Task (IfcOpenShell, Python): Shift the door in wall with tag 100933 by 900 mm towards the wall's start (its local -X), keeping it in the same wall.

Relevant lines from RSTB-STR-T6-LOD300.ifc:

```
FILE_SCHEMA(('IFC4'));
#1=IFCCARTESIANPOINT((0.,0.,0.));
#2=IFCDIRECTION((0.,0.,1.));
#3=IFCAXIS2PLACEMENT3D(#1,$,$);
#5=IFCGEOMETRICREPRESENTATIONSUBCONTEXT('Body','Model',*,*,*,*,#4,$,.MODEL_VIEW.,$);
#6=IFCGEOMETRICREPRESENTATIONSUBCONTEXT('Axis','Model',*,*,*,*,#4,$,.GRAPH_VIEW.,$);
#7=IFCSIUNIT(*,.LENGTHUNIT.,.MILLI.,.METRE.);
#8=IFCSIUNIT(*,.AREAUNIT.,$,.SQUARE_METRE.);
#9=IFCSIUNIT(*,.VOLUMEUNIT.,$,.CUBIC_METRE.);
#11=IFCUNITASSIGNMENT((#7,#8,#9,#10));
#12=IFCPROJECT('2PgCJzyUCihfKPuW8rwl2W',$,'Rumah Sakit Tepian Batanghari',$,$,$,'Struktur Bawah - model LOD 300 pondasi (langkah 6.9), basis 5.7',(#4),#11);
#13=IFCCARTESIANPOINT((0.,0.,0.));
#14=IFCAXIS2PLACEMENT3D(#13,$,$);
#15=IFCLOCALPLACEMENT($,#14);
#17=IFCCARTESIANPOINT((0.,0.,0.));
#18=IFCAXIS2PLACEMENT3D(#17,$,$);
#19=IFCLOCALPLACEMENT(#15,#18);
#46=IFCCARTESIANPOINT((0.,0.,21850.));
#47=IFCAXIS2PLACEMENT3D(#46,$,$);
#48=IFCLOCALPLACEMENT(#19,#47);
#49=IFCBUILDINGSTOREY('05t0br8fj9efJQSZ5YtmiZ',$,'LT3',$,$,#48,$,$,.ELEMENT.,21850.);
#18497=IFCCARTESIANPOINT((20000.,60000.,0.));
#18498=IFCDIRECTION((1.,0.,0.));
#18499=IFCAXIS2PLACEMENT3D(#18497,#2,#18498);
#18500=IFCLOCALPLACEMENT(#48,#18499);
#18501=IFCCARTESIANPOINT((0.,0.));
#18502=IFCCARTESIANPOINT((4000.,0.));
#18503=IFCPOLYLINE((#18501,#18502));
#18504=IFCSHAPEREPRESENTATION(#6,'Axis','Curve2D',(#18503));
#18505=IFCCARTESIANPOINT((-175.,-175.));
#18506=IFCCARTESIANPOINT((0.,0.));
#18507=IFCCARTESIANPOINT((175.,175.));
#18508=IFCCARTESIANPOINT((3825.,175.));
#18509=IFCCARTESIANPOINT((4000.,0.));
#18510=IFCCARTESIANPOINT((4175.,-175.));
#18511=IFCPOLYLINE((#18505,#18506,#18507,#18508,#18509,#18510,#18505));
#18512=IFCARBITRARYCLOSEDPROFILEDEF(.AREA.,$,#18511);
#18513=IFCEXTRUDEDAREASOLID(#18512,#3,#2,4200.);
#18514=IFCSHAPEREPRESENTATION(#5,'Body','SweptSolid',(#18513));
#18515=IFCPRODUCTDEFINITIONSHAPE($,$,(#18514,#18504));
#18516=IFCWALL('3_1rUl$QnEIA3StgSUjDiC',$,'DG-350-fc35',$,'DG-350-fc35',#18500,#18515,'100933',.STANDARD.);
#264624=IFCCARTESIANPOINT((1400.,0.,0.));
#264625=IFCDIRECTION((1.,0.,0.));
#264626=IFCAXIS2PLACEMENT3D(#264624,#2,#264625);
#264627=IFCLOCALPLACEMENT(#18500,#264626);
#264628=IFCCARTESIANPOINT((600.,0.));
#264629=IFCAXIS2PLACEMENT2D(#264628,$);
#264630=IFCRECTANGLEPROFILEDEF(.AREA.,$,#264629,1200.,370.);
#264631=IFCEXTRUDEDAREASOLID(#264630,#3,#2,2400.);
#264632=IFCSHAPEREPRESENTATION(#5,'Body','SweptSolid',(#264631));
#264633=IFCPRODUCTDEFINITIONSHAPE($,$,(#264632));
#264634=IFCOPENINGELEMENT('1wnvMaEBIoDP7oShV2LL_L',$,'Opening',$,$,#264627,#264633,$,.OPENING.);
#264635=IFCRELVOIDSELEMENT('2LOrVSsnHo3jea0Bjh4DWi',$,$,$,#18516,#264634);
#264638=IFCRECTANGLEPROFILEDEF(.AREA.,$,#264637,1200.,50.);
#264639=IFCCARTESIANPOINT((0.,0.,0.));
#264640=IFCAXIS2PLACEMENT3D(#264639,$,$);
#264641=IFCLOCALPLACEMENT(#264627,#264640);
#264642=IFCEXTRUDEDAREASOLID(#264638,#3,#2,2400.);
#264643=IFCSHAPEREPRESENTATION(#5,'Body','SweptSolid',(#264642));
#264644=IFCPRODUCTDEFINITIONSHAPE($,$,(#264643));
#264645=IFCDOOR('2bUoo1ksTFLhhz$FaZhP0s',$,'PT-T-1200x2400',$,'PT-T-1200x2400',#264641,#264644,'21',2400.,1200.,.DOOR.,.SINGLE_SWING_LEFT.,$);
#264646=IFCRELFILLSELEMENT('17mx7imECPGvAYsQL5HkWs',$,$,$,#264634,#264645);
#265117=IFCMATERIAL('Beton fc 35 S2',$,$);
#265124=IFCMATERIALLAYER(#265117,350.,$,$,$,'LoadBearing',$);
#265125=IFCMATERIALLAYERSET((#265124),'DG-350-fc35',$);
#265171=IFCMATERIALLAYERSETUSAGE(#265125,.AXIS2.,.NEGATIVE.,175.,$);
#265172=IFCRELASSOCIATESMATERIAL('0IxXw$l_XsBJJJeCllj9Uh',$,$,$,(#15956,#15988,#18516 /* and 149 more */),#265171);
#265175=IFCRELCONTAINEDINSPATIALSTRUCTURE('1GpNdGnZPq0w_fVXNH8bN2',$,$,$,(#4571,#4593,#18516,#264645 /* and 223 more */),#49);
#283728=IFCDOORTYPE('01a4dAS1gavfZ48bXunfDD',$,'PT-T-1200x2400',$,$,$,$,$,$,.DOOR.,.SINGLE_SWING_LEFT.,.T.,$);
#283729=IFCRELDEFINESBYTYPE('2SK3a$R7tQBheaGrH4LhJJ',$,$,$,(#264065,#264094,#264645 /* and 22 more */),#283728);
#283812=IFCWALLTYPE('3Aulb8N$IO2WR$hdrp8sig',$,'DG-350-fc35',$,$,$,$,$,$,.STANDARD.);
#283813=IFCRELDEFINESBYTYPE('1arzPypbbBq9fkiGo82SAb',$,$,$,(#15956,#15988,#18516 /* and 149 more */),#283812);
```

```python
import ifcopenshell
import ifcopenshell.api.geometry
import ifcopenshell.util.placement
import ifcopenshell.util.unit

model = ifcopenshell.open("RSTB-STR-T6-LOD300.ifc")
unit_scale = ifcopenshell.util.unit.calculate_unit_scale(model)

door = model.by_id(264645)
opening = door.FillsVoids[0].RelatingOpeningElement
wall = opening.VoidsElements[0].RelatingBuildingElement

wall_matrix = ifcopenshell.util.placement.get_local_placement(wall.ObjectPlacement)
shift = wall_matrix[:3, 0] * -0.9 / unit_scale
before = ifcopenshell.util.placement.get_local_placement(door.ObjectPlacement)[:3, 3].copy()

# The door is placed relative to its opening, so it follows when the opening moves.
matrix = ifcopenshell.util.placement.get_local_placement(opening.ObjectPlacement)
matrix[:3, 3] += shift
ifcopenshell.api.geometry.edit_object_placement(
    model, product=opening, matrix=matrix, is_si=False, should_transform_children=True
)

after = ifcopenshell.util.placement.get_local_placement(door.ObjectPlacement)[:3, 3]
print("door moved by", (after - before).round(3) + 0.0)

model.write("RSTB-STR-T6-LOD300_v2.ifc")
```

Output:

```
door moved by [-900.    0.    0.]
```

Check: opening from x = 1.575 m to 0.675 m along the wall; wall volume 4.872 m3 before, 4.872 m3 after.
